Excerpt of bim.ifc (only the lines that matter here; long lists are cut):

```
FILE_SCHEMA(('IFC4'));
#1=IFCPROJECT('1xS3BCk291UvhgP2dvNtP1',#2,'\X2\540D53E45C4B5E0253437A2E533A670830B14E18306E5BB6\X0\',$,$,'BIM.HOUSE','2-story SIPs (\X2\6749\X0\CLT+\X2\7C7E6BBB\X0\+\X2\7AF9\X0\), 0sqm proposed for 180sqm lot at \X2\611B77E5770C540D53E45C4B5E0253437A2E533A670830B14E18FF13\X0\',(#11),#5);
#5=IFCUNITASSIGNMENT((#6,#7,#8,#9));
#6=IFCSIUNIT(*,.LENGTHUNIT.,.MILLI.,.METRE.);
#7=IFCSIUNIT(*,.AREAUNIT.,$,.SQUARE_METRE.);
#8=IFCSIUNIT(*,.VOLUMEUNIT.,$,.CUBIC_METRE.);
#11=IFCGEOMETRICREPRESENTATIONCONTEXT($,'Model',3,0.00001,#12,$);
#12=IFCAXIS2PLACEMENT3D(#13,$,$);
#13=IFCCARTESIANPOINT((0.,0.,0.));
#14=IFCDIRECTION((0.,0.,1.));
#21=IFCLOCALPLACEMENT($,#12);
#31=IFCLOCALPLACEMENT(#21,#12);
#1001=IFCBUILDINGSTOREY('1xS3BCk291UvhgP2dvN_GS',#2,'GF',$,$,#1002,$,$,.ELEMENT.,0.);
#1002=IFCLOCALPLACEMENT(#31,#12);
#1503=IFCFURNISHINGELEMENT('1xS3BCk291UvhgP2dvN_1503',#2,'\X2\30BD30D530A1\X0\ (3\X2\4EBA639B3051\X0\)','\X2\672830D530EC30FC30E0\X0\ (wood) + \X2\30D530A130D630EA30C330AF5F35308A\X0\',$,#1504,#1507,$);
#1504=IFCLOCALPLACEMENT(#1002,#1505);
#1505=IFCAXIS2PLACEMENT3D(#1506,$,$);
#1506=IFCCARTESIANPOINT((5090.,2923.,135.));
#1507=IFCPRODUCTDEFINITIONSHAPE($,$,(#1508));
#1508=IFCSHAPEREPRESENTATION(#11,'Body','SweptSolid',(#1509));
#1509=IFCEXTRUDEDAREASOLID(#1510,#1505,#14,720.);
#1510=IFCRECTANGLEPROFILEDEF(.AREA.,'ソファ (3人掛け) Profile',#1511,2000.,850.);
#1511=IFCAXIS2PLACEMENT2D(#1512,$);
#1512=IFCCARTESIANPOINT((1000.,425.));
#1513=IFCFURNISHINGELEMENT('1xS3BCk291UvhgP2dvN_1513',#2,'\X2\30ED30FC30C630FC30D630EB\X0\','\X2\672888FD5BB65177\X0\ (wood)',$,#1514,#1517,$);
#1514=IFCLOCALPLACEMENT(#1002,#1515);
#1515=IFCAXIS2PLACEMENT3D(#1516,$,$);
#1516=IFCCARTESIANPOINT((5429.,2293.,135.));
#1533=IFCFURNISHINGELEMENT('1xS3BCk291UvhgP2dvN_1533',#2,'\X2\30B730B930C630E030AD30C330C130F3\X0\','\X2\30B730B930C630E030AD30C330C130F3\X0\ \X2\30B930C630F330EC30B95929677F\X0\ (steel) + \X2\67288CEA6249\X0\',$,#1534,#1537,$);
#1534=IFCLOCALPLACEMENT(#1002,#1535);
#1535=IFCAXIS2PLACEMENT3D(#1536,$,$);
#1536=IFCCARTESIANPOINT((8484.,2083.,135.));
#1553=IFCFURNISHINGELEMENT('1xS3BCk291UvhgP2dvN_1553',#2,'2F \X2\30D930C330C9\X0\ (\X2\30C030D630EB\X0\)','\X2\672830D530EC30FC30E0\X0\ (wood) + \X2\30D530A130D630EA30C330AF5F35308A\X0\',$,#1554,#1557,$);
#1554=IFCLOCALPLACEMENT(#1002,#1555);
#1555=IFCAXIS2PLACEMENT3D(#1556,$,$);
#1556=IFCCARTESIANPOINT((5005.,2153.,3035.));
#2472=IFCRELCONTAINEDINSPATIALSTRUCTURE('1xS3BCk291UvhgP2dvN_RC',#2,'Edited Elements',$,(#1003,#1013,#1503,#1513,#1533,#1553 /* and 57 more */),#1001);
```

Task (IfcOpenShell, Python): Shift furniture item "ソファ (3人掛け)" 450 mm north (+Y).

```python
import ifcopenshell
import ifcopenshell.api.geometry
import ifcopenshell.util.placement
import ifcopenshell.util.unit

model = ifcopenshell.open("bim.ifc")
unit_scale = ifcopenshell.util.unit.calculate_unit_scale(model)

item = model.by_guid("1xS3BCk291UvhgP2dvN_1503")
matrix = ifcopenshell.util.placement.get_local_placement(item.ObjectPlacement)
matrix[1, 3] += 0.45 / unit_scale
ifcopenshell.api.geometry.edit_object_placement(model, product=item, matrix=matrix, is_si=False)

print(ifcopenshell.util.placement.get_local_placement(item.ObjectPlacement).round(3) + 0.0)

model.write("bim_v2.ifc")
```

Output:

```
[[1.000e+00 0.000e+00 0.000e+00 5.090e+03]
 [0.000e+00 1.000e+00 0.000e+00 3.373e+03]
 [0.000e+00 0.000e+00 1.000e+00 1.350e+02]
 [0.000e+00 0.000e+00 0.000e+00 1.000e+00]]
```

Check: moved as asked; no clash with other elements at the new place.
